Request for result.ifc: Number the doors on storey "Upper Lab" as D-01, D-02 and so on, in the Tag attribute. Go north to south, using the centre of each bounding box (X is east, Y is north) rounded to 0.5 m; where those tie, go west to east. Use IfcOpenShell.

First a look at what the model holds.

```python
import ifcopenshell
import ifcopenshell.util.element
import ifcopenshell.util.placement

model = ifcopenshell.open("result.ifc")
print(model.schema)
storey = next(s for s in model.by_type("IfcBuildingStorey") if s.Name == "Upper Lab")
doors = [e for e in ifcopenshell.util.element.get_decomposition(storey) if e.is_a("IfcDoor")]
for e in sorted(doors, key=lambda e: e.id()):
    origin = ifcopenshell.util.placement.get_local_placement(e.ObjectPlacement)[:3, 3]
    print(e.id(), e.Tag, e.Name, origin.round(2) + 0.0, sep=" | ")
```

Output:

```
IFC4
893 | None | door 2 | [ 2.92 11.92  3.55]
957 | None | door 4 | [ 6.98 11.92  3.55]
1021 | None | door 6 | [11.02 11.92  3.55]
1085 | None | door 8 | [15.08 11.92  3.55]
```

```python
import ifcopenshell
import ifcopenshell.geom
import ifcopenshell.util.element
import ifcopenshell.util.shape

model = ifcopenshell.open("result.ifc")
settings = ifcopenshell.geom.settings()
settings.set("use-world-coords", True)


def centre(element):
    shape = ifcopenshell.geom.create_shape(settings, element)
    return ifcopenshell.util.shape.get_bbox_centroid(shape.geometry)


storey = next(s for s in model.by_type("IfcBuildingStorey") if s.Name == "Upper Lab")
doors = [e for e in ifcopenshell.util.element.get_decomposition(storey) if e.is_a("IfcDoor")]

# Insertion points can sit at a corner or the storey origin, so sort by the geometry (in metres).
centres = {e: centre(e) for e in doors}
doors.sort(key=lambda e: (-round(centres[e][1] / 0.5), centres[e][0]))

for i, e in enumerate(doors, start=1):
    number = f"D-{i:02d}"
    e.Tag = number
    print(e.id(), number)

model.write("result_rev.ifc")
```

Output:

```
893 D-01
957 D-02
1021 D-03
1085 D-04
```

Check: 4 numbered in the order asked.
